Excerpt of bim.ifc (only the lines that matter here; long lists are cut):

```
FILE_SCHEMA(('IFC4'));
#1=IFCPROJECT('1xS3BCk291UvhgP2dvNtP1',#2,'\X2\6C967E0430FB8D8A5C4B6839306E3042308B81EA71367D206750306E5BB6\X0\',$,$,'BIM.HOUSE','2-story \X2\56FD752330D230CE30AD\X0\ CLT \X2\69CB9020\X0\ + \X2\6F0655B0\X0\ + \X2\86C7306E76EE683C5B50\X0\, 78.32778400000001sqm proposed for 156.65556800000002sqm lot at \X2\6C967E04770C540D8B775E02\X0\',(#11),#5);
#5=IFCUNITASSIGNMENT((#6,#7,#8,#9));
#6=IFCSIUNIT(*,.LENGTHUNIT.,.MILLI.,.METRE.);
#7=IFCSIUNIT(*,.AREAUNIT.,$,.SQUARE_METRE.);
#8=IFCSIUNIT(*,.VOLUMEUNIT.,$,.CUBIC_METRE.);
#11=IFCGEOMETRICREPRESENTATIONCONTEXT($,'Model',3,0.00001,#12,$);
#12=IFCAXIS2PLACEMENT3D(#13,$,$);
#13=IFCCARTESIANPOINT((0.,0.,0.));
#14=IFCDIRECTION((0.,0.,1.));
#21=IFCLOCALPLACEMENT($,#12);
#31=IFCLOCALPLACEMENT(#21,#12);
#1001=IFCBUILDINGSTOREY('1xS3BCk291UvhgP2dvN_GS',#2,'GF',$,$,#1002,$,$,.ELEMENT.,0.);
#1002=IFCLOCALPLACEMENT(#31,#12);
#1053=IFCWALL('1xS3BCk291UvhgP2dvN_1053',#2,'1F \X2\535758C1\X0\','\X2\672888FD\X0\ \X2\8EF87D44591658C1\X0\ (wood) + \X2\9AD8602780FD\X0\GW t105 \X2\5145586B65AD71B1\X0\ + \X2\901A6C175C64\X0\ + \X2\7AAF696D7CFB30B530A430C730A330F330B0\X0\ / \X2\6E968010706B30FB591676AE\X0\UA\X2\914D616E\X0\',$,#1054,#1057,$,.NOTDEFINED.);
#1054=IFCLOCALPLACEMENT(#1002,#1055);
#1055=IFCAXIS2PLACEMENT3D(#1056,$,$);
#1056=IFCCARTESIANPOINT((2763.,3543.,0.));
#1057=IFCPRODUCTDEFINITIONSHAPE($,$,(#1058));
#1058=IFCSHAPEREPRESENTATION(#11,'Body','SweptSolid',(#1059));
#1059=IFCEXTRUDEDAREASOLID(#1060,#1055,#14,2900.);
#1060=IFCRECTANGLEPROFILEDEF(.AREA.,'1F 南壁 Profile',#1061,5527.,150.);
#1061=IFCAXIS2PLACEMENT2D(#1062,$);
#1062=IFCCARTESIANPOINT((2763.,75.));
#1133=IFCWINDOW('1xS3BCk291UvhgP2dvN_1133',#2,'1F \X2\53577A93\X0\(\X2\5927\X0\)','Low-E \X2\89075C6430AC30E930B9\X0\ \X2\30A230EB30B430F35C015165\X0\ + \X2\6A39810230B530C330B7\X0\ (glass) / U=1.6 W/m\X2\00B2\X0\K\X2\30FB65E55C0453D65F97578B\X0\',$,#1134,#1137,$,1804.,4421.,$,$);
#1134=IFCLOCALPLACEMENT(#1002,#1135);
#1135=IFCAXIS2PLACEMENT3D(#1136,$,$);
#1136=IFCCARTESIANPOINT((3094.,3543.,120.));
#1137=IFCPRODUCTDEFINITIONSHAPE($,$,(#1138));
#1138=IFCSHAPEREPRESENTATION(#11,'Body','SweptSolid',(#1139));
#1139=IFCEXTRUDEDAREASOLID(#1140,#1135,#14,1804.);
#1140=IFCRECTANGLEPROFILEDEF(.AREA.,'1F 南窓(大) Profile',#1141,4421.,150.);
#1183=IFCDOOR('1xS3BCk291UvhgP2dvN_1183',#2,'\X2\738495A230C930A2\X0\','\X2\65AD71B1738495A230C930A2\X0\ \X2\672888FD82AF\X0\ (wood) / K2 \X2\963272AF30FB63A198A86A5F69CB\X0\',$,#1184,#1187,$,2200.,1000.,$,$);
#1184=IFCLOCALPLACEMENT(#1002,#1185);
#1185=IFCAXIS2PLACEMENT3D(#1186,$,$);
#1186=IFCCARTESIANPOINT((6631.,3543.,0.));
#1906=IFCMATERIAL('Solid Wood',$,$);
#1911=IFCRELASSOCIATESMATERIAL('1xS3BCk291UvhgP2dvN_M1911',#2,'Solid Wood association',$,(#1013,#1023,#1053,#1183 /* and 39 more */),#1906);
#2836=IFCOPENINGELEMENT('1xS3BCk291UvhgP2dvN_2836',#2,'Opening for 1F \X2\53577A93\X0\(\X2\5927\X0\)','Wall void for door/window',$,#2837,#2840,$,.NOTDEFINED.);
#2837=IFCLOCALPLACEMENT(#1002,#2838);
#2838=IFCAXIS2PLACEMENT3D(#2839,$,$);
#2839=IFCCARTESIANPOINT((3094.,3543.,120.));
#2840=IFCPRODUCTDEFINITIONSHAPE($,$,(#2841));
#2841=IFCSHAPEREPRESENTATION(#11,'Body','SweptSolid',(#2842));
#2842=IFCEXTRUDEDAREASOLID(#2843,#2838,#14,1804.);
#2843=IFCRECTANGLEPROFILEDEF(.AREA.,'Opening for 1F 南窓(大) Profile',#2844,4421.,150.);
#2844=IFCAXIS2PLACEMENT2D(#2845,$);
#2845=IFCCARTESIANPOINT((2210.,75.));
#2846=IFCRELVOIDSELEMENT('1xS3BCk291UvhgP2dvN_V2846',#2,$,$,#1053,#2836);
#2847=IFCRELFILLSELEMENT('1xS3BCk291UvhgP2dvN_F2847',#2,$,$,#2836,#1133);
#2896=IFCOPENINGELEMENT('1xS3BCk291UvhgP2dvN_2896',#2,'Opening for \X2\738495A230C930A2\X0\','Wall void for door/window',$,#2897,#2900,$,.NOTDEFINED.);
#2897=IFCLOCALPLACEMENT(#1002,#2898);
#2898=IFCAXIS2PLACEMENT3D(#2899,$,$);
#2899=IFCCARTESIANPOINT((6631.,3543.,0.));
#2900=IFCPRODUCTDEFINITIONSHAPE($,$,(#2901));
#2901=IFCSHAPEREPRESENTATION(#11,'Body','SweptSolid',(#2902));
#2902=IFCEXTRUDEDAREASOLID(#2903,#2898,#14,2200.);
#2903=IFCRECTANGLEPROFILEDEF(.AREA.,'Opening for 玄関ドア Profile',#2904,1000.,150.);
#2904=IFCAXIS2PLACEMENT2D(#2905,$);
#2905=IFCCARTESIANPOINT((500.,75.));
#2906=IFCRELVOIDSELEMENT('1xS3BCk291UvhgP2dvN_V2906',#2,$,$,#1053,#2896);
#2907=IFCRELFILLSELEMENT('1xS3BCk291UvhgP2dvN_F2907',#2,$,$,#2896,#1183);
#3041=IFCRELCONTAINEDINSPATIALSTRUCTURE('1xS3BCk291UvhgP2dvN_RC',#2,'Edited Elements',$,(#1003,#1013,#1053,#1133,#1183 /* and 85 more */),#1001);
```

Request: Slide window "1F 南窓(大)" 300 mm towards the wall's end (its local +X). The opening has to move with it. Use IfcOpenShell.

```python
import ifcopenshell
import ifcopenshell.api.geometry
import ifcopenshell.util.placement
import ifcopenshell.util.unit

model = ifcopenshell.open("bim.ifc")
unit_scale = ifcopenshell.util.unit.calculate_unit_scale(model)

window = model.by_id(1133)
opening = window.FillsVoids[0].RelatingOpeningElement
wall = opening.VoidsElements[0].RelatingBuildingElement

wall_matrix = ifcopenshell.util.placement.get_local_placement(wall.ObjectPlacement)
shift = wall_matrix[:3, 0] * 0.3 / unit_scale
before = ifcopenshell.util.placement.get_local_placement(window.ObjectPlacement)[:3, 3].copy()

# The window is not placed relative to its opening, so move both.
for product in (opening, window):
    matrix = ifcopenshell.util.placement.get_local_placement(product.ObjectPlacement)
    matrix[:3, 3] += shift
    ifcopenshell.api.geometry.edit_object_placement(model, product=product, matrix=matrix, is_si=False)

after = ifcopenshell.util.placement.get_local_placement(window.ObjectPlacement)[:3, 3]
print("window moved by", (after - before).round(3) + 0.0)

model.write("bim_edited.ifc")
```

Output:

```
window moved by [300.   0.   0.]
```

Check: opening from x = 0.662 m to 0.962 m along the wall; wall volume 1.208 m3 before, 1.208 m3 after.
